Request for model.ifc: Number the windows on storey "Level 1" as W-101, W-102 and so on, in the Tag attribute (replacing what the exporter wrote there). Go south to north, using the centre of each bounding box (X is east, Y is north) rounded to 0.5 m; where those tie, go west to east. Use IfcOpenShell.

First a look at what the model holds.

```python
import ifcopenshell
import ifcopenshell.util.element
import ifcopenshell.util.placement

model = ifcopenshell.open("model.ifc")
print(model.schema)
storey = next(s for s in model.by_type("IfcBuildingStorey") if s.Name == "Level 1")
windows = [e for e in ifcopenshell.util.element.get_decomposition(storey) if e.is_a("IfcWindow")]
for e in sorted(windows, key=lambda e: e.id()):
    origin = ifcopenshell.util.placement.get_local_placement(e.ObjectPlacement)[:3, 3]
    print(e.id(), e.Tag, e.Name, origin.round(2) + 0.0, sep=" | ")
```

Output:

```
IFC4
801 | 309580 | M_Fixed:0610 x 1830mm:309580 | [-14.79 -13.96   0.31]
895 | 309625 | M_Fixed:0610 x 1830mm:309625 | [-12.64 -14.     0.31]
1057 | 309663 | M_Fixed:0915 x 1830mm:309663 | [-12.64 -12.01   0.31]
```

```python
import ifcopenshell
import ifcopenshell.geom
import ifcopenshell.util.element
import ifcopenshell.util.shape

model = ifcopenshell.open("model.ifc")
settings = ifcopenshell.geom.settings()
settings.set("use-world-coords", True)


def centre(element):
    shape = ifcopenshell.geom.create_shape(settings, element)
    return ifcopenshell.util.shape.get_bbox_centroid(shape.geometry)


storey = next(s for s in model.by_type("IfcBuildingStorey") if s.Name == "Level 1")
windows = [e for e in ifcopenshell.util.element.get_decomposition(storey) if e.is_a("IfcWindow")]

# Insertion points can sit at a corner or the storey origin, so sort by the geometry (in metres).
centres = {e: centre(e) for e in windows}
windows.sort(key=lambda e: (round(centres[e][1] / 0.5), centres[e][0]))

for i, e in enumerate(windows, start=1):
    number = f"W-1{i:02d}"
    e.Tag = number
    print(e.id(), number)

model.write("model_updated.ifc")
```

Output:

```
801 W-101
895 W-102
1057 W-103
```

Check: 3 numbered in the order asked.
